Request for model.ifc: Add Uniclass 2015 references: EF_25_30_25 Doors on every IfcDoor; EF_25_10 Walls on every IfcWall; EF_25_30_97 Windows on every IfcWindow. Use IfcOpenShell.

First a look at what the model holds.

```python
import ifcopenshell

model = ifcopenshell.open("model.ifc")
print(model.schema)
print("classifications:", [c.Name for c in model.by_type("IfcClassification")])
for ifc_class in ("IfcDoor", "IfcRoof", "IfcStair", "IfcWall", "IfcWindow"):
    print(ifc_class, len(model.by_type(ifc_class)))
```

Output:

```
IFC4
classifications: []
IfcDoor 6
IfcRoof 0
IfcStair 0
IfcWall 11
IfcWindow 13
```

```python
import ifcopenshell
import ifcopenshell.api.classification

model = ifcopenshell.open("model.ifc")

system = ifcopenshell.api.classification.add_classification(model, classification="Uniclass 2015")

codes = {
    "IfcDoor": ("EF_25_30_25", "Doors"),
    "IfcWall": ("EF_25_10", "Walls"),
    "IfcWindow": ("EF_25_30_97", "Windows"),
}
for ifc_class, (code, name) in codes.items():
    products = model.by_type(ifc_class)
    ifcopenshell.api.classification.add_reference(
        model, products=products, classification=system, identification=code, name=name
    )
    print(code, len(products))

model.write("model_rev.ifc")
```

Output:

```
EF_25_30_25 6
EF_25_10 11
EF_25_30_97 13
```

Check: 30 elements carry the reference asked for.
